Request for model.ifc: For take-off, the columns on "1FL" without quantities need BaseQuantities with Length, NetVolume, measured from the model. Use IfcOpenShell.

First a look at what the model holds.

```python
import ifcopenshell
import ifcopenshell.util.element
import ifcopenshell.util.unit

model = ifcopenshell.open("model.ifc")
print(model.schema)
for unit_type in ("LENGTHUNIT", "AREAUNIT", "VOLUMEUNIT"):
    print(unit_type, ifcopenshell.util.unit.calculate_unit_scale(model, unit_type))
storey = next(s for s in model.by_type("IfcBuildingStorey") if s.Name == "1FL")
columns = [e for e in ifcopenshell.util.element.get_decomposition(storey) if e.is_a("IfcColumn")]
for e in sorted(columns, key=lambda e: e.id()):
    print(e.id(), e.is_a(), e.Name, list(ifcopenshell.util.element.get_psets(e, qtos_only=True)), sep=" | ")
```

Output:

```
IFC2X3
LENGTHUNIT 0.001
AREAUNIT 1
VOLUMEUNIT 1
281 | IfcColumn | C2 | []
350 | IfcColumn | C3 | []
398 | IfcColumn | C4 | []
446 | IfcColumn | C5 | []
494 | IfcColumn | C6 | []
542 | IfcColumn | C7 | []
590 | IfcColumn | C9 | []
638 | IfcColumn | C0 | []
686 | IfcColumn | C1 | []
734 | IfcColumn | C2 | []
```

```python
import ifcopenshell
import ifcopenshell.api.pset
import ifcopenshell.geom
import ifcopenshell.util.element
import ifcopenshell.util.shape
import ifcopenshell.util.unit

model = ifcopenshell.open("model.ifc")
unit_scale = ifcopenshell.util.unit.calculate_unit_scale(model)
volume_scale = ifcopenshell.util.unit.calculate_unit_scale(model, "VOLUMEUNIT")
settings = ifcopenshell.geom.settings()

storey = next(s for s in model.by_type("IfcBuildingStorey") if s.Name == "1FL")
columns = [e for e in ifcopenshell.util.element.get_decomposition(storey) if e.is_a("IfcColumn")]

for e in sorted(columns, key=lambda e: e.id()):
    if ifcopenshell.util.element.get_psets(e, qtos_only=True, should_inherit=False):
        continue
    # Geometry comes back in metres, in the element's own axes.
    shape = ifcopenshell.geom.create_shape(settings, e)
    values = {
        "Length": ifcopenshell.util.shape.get_z(shape.geometry) / unit_scale,
        "NetVolume": ifcopenshell.util.shape.get_volume(shape.geometry) / volume_scale,
    }
    qto = ifcopenshell.api.pset.add_qto(model, product=e, name="BaseQuantities")
    ifcopenshell.api.pset.edit_qto(model, qto=qto, properties=values)
    print(e.id(), {k: round(v, 3) for k, v in values.items()})

model.write("model_rev.ifc")
```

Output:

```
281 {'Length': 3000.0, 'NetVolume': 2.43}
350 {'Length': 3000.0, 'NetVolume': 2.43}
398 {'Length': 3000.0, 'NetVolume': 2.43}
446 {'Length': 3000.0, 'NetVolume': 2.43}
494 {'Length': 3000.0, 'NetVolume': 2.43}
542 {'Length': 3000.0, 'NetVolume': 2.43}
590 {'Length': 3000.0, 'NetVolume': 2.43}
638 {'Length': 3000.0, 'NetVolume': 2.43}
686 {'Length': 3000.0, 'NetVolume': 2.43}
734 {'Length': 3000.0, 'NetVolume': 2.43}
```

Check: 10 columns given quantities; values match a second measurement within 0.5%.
